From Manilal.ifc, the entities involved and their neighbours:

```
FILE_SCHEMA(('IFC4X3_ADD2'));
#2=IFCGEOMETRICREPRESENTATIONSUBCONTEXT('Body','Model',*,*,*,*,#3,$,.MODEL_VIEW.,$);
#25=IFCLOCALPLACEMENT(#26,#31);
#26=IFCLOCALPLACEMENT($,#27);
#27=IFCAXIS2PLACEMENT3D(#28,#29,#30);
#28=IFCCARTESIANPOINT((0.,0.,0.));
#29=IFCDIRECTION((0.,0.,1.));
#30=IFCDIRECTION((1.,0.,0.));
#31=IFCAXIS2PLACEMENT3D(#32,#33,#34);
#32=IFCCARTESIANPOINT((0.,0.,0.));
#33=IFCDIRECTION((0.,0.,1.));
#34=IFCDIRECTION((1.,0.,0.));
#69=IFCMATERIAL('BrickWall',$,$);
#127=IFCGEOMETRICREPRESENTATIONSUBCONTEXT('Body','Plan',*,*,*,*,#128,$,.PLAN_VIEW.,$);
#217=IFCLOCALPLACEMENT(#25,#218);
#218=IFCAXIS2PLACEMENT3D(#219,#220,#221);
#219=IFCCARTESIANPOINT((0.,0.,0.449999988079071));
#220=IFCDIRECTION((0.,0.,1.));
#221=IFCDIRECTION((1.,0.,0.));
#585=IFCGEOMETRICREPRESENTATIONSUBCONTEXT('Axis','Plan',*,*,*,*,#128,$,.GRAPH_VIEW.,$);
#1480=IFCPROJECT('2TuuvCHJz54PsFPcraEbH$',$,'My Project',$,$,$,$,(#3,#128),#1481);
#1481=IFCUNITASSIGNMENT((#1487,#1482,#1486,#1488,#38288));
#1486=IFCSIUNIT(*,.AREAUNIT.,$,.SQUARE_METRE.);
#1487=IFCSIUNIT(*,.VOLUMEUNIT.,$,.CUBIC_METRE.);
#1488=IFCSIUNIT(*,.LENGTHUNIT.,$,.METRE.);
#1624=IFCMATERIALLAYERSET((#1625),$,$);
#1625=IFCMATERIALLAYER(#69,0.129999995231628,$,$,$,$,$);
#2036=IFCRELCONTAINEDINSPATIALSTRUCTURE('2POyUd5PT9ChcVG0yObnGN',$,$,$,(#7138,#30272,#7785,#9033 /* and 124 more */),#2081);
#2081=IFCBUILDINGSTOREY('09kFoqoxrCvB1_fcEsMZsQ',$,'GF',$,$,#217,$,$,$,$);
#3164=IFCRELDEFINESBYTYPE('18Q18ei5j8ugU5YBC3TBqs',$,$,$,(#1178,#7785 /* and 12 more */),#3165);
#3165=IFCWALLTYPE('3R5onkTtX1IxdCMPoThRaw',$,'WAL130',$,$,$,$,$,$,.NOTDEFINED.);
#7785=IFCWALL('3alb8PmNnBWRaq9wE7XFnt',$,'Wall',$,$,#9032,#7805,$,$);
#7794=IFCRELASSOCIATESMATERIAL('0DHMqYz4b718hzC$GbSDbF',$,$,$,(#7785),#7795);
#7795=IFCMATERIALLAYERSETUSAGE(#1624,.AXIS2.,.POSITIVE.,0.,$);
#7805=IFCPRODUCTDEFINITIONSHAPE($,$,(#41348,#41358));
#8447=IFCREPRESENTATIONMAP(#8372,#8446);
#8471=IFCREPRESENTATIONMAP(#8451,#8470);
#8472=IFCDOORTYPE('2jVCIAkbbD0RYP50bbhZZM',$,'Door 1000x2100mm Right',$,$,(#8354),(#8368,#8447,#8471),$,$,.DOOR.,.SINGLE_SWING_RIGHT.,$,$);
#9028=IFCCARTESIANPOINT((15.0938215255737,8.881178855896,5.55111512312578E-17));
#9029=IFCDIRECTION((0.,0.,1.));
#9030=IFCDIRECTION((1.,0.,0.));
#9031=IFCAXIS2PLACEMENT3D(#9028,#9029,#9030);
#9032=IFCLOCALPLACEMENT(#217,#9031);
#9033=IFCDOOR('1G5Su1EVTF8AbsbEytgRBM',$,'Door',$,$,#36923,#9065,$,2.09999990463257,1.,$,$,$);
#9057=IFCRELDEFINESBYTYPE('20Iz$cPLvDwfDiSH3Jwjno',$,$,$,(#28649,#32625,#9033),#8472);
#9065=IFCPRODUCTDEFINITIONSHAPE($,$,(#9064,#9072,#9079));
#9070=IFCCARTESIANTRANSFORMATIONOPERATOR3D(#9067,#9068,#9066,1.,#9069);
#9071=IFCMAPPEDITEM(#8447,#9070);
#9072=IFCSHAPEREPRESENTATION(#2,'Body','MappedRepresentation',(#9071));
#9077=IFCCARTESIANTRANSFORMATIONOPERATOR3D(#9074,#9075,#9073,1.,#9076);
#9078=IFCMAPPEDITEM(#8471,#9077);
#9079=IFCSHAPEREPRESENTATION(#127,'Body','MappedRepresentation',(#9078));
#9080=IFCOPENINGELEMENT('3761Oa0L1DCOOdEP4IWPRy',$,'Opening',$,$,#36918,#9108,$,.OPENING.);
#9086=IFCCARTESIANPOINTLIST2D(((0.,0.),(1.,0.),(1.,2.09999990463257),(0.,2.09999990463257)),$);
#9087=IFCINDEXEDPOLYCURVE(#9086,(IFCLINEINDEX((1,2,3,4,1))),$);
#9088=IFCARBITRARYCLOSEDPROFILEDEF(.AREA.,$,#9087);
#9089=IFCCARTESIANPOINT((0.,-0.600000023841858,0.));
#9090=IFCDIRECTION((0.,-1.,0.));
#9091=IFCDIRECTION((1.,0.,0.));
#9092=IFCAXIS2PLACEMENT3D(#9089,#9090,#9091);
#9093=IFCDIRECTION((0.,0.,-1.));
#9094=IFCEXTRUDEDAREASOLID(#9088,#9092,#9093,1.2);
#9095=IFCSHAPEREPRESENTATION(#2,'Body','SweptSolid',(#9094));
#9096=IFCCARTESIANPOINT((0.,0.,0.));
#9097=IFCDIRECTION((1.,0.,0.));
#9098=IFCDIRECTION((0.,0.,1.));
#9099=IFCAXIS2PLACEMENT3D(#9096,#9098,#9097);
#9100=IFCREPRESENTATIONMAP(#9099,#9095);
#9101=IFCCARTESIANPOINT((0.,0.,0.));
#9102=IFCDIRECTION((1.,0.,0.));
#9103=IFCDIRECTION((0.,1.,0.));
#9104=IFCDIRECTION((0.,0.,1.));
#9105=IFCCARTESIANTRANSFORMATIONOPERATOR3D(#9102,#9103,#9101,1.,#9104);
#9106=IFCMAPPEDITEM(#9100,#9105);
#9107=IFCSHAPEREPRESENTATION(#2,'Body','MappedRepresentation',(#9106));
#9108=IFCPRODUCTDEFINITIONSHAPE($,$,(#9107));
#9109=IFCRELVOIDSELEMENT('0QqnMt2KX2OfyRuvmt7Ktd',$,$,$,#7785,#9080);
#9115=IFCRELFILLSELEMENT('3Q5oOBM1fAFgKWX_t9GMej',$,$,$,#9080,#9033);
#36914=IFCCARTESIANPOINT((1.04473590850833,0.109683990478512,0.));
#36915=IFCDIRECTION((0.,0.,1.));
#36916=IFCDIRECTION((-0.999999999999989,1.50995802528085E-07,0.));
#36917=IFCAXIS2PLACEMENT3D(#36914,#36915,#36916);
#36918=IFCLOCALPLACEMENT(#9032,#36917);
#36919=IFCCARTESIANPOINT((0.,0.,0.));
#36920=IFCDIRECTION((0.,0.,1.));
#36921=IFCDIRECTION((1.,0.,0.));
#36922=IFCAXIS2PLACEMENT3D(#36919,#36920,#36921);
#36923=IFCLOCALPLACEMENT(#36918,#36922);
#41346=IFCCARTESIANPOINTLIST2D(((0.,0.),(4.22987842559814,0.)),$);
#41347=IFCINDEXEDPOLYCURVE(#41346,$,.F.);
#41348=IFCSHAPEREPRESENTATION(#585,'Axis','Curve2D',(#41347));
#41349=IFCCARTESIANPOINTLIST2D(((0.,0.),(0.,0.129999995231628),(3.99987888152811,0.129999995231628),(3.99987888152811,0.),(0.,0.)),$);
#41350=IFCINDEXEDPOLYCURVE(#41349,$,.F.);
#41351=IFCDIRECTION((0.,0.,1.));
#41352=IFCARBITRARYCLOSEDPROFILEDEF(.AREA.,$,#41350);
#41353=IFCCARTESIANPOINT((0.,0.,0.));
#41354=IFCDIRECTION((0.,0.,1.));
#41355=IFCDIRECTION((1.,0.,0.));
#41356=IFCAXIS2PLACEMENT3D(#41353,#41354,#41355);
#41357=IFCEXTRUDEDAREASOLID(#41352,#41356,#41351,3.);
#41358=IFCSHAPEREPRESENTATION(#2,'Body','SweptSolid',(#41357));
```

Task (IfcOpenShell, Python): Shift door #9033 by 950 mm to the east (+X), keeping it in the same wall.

```python
import ifcopenshell
import ifcopenshell.api.geometry
import ifcopenshell.util.placement
import ifcopenshell.util.unit

model = ifcopenshell.open("Manilal.ifc")
unit_scale = ifcopenshell.util.unit.calculate_unit_scale(model)

door = model.by_id(9033)
opening = door.FillsVoids[0].RelatingOpeningElement
wall = opening.VoidsElements[0].RelatingBuildingElement

wall_matrix = ifcopenshell.util.placement.get_local_placement(wall.ObjectPlacement)
shift = wall_matrix[:3, 0] * 0.95 / unit_scale
before = ifcopenshell.util.placement.get_local_placement(door.ObjectPlacement)[:3, 3].copy()

# The door is placed relative to its opening, so it follows when the opening moves.
matrix = ifcopenshell.util.placement.get_local_placement(opening.ObjectPlacement)
matrix[:3, 3] += shift
ifcopenshell.api.geometry.edit_object_placement(
    model, product=opening, matrix=matrix, is_si=False, should_transform_children=True
)

after = ifcopenshell.util.placement.get_local_placement(door.ObjectPlacement)[:3, 3]
print("door moved by", (after - before).round(3) + 0.0)

model.write("Manilal_v2.ifc")
```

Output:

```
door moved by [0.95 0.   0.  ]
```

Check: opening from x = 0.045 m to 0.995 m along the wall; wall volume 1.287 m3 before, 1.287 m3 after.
